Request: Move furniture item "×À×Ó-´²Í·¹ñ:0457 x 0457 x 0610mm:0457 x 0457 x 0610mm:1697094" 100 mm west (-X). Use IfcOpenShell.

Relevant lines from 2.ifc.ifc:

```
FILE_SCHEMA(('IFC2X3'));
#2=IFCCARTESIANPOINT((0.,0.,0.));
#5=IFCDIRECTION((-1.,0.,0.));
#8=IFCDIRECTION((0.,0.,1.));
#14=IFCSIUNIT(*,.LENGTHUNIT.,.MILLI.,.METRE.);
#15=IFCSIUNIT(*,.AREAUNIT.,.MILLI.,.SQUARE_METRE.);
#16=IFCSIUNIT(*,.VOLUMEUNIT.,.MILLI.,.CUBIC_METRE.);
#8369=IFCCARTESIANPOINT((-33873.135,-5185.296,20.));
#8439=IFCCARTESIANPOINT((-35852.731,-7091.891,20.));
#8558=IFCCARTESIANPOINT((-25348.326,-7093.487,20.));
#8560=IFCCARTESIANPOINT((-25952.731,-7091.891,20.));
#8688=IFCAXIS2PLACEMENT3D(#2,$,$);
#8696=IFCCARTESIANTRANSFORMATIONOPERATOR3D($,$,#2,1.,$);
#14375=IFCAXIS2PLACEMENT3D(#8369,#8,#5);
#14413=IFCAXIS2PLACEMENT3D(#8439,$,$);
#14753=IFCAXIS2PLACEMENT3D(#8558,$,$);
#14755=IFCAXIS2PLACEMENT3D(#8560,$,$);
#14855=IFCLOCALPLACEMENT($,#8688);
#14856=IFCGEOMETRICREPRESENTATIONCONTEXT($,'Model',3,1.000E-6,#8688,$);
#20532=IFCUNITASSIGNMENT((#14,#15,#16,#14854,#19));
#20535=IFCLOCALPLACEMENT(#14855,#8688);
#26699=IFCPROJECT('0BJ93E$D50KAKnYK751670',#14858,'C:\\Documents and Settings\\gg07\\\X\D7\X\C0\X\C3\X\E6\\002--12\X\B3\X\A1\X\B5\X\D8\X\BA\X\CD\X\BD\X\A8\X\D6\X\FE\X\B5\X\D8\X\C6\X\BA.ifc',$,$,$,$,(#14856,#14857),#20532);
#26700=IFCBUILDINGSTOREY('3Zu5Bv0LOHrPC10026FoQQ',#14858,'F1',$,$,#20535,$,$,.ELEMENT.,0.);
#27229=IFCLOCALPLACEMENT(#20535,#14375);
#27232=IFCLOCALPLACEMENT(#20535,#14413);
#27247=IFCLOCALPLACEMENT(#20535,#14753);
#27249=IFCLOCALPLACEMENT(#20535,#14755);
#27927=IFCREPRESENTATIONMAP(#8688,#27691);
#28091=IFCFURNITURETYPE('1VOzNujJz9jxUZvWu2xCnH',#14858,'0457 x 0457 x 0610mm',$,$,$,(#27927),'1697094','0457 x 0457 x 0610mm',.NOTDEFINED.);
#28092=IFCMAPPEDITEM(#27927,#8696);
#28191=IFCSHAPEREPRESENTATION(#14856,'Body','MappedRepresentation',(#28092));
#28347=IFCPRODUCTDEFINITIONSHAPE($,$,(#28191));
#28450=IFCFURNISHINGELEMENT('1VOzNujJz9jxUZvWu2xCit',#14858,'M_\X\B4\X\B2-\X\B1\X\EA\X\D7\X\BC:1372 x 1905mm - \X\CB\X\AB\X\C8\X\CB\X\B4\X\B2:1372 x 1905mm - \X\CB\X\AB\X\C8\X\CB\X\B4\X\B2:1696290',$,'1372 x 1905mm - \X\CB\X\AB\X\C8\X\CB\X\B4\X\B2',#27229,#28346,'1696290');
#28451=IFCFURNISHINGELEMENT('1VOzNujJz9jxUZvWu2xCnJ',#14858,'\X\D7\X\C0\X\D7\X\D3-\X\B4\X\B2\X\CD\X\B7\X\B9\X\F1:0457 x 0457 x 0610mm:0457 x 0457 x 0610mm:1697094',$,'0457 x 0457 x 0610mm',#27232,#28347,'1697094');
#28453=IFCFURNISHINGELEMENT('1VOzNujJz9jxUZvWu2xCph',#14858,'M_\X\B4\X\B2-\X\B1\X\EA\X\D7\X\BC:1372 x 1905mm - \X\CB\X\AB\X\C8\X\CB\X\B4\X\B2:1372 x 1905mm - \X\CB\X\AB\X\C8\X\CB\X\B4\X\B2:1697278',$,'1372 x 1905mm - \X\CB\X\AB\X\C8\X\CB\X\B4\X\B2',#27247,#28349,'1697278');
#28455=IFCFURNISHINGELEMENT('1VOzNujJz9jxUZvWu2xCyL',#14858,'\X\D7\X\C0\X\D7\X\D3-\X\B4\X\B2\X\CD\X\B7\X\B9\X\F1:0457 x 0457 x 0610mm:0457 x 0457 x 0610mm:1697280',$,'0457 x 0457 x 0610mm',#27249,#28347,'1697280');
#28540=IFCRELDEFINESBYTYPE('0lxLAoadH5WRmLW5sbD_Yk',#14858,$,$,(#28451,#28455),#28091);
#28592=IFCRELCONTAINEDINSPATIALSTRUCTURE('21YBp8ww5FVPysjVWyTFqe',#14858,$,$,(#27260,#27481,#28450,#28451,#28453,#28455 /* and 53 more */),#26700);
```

```python
import ifcopenshell
import ifcopenshell.api.geometry
import ifcopenshell.util.placement

model = ifcopenshell.open("2.ifc.ifc")

item = model.by_id(28451)
matrix = ifcopenshell.util.placement.get_local_placement(item.ObjectPlacement)
matrix[0, 3] -= 100.0
ifcopenshell.api.geometry.edit_object_placement(model, product=item, matrix=matrix, is_si=False)

print(ifcopenshell.util.placement.get_local_placement(item.ObjectPlacement).round(3) + 0.0)

model.write("2.ifc-out.ifc")
```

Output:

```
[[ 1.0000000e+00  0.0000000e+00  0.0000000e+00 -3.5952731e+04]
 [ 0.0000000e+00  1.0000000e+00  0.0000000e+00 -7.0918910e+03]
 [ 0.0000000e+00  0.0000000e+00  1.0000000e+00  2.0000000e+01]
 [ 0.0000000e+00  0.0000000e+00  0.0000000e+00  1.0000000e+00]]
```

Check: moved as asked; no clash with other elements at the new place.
